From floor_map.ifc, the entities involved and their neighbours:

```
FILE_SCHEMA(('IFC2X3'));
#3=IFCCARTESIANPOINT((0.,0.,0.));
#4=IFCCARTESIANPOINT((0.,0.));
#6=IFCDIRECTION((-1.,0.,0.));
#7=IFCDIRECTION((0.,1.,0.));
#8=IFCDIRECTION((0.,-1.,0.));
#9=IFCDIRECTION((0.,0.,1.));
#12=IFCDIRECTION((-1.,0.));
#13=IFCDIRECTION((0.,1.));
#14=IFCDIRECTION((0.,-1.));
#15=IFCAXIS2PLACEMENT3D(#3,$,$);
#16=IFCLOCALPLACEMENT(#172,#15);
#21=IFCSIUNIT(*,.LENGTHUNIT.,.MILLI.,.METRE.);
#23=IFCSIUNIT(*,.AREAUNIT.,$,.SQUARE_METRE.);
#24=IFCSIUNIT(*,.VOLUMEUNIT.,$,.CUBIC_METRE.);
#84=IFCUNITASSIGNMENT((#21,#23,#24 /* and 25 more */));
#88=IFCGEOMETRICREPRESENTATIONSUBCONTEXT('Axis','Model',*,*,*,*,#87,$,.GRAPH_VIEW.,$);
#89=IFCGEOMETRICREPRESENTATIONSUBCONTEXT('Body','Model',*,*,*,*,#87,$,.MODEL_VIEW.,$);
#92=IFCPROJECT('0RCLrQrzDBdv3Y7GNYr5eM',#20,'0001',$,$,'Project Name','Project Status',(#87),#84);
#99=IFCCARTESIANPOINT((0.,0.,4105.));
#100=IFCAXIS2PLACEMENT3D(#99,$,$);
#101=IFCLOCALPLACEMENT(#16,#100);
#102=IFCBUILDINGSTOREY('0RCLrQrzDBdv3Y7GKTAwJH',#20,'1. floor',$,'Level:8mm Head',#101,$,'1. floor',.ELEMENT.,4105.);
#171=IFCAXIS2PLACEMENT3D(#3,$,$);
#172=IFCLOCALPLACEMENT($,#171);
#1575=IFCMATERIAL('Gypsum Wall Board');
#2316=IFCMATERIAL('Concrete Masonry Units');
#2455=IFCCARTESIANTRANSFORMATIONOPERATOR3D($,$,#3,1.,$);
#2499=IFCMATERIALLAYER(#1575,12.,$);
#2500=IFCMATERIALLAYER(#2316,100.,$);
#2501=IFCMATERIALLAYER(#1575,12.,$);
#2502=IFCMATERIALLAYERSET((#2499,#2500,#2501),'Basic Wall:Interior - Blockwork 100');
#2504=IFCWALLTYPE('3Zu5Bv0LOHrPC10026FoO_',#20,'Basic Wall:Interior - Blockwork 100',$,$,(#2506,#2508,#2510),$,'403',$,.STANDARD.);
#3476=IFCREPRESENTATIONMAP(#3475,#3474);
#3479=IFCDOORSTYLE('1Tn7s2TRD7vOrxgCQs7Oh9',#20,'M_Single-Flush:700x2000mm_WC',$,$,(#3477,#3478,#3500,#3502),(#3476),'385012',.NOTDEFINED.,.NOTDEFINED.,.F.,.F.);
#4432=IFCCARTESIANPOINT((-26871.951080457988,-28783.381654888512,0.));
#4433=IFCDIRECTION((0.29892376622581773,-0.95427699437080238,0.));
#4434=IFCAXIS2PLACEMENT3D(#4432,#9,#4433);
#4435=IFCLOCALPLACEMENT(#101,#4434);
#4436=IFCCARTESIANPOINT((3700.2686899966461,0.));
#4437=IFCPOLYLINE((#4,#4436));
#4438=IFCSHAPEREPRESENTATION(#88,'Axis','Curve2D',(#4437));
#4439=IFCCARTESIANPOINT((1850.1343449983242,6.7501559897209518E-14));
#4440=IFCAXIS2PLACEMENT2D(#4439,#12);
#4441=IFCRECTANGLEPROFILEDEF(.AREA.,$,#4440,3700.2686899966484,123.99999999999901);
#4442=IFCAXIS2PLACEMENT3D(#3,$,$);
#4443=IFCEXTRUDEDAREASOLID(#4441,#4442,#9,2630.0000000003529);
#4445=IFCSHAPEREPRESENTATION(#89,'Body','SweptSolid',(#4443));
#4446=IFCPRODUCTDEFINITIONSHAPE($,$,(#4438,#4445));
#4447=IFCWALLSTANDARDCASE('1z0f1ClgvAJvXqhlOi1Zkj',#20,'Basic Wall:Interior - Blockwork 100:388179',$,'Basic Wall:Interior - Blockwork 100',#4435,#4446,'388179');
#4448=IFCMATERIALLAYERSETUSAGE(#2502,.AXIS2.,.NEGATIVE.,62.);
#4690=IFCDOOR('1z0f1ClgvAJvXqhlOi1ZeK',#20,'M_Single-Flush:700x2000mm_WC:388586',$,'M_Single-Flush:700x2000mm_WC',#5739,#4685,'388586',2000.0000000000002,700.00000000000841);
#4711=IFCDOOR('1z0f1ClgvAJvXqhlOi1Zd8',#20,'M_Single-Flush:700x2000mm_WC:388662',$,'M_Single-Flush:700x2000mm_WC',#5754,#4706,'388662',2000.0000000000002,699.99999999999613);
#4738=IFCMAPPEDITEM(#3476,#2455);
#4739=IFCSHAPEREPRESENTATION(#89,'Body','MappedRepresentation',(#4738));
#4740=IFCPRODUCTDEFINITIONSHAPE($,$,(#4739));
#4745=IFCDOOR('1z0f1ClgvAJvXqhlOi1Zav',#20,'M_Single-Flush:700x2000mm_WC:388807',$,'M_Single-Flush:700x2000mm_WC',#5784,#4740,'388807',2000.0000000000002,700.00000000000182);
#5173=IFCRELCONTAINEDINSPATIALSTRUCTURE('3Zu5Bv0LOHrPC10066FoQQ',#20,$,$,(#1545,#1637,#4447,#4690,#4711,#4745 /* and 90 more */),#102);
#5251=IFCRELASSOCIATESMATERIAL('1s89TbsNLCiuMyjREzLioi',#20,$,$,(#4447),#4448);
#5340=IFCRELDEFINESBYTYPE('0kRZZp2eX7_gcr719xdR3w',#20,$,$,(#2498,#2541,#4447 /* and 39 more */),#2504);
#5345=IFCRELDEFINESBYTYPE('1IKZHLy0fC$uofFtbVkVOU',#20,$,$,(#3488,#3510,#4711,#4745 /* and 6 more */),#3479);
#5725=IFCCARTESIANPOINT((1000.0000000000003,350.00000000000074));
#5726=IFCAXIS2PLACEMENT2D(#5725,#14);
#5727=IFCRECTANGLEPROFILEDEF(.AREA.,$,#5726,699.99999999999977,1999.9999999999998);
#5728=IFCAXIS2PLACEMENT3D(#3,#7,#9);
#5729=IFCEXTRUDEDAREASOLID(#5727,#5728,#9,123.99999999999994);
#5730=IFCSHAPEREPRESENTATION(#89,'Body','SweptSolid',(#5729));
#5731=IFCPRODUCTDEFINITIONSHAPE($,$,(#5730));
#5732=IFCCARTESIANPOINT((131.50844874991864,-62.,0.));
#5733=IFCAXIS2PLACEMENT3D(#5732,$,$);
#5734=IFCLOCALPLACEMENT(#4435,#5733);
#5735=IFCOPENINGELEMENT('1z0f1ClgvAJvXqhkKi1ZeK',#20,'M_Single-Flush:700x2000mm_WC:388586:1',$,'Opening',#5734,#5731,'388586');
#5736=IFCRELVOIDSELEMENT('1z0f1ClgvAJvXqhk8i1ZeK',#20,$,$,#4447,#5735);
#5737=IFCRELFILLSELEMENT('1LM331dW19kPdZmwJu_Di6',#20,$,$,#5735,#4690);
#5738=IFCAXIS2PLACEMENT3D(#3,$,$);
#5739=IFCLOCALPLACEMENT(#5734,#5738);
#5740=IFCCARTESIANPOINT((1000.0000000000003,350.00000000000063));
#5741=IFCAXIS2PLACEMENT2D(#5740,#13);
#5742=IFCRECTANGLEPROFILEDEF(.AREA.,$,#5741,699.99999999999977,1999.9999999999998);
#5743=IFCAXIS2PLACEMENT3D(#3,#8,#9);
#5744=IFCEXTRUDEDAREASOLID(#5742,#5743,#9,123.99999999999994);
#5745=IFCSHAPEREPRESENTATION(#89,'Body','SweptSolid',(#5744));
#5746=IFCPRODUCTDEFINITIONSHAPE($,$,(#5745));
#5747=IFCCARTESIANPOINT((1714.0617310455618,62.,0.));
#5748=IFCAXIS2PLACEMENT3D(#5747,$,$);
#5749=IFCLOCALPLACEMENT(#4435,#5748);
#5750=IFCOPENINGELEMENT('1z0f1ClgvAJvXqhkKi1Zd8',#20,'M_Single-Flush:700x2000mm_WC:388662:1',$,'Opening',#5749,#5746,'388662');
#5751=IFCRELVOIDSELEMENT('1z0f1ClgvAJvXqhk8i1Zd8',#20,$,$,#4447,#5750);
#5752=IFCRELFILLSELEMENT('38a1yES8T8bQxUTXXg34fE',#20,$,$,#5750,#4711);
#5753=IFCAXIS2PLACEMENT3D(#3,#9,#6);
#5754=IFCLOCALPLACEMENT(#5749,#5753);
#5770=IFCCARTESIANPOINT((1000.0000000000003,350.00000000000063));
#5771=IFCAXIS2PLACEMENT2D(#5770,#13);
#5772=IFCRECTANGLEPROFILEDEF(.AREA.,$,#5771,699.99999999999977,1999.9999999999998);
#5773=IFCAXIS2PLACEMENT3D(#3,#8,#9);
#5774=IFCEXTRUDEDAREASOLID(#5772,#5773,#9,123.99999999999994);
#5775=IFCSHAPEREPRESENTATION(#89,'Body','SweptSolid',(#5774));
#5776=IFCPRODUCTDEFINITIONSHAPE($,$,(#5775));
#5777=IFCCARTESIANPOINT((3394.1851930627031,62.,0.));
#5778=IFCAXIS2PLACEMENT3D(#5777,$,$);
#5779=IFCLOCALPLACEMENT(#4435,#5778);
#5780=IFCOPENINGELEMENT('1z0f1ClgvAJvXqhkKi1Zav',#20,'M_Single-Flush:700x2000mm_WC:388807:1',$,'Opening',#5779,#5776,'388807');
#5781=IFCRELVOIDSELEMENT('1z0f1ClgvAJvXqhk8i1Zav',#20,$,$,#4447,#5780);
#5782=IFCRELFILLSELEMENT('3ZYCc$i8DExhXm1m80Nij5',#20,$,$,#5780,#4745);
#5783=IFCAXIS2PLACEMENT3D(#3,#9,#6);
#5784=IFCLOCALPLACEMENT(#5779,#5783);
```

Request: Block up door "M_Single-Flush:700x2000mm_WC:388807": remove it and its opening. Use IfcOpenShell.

```python
import ifcopenshell
import ifcopenshell.api.feature
import ifcopenshell.api.root
import ifcopenshell.geom
import ifcopenshell.util.shape

model = ifcopenshell.open("floor_map.ifc")
settings = ifcopenshell.geom.settings()


def volume(element):
    """Net volume in cubic metres, openings subtracted."""
    shape = ifcopenshell.geom.create_shape(settings, element)
    return ifcopenshell.util.shape.get_volume(shape.geometry)


door = model.by_guid("1z0f1ClgvAJvXqhlOi1Zav")
opening = door.FillsVoids[0].RelatingOpeningElement
wall = opening.VoidsElements[0].RelatingBuildingElement
before = volume(wall)

ifcopenshell.api.root.remove_product(model, product=door)
ifcopenshell.api.feature.remove_feature(model, feature=opening)

after = volume(wall)

print(f"wall volume {before:.3f} -> {after:.3f} m3")

model.write("floor_map-out.ifc")
```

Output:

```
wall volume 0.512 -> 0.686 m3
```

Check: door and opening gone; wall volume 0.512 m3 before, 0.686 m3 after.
